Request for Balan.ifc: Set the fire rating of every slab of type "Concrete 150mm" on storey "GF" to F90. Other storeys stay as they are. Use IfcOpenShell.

First a look at what the model holds.

```python
import ifcopenshell
import ifcopenshell.util.element

model = ifcopenshell.open("Balan.ifc")
print(model.schema)
storey = next(s for s in model.by_type("IfcBuildingStorey") if s.Name == "GF")
slabs = [e for e in ifcopenshell.util.element.get_decomposition(storey) if e.is_a("IfcSlab")]
seen = {}
for e in slabs:
    element_type = ifcopenshell.util.element.get_type(e)
    key = (element_type.Name if element_type != e and element_type else None, ifcopenshell.util.element.get_pset(e, "Pset_SlabCommon", "FireRating"))
    seen[key] = seen.get(key, 0) + 1
for (name, value), count in sorted(seen.items(), key=str):
    print(count, "x", name, "|", value)
```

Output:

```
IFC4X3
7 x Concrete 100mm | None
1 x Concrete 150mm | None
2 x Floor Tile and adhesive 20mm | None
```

```python
import ifcopenshell
import ifcopenshell.api.pset
import ifcopenshell.util.element

model = ifcopenshell.open("Balan.ifc")

storey = next(s for s in model.by_type("IfcBuildingStorey") if s.Name == "GF")
slabs = [e for e in ifcopenshell.util.element.get_decomposition(storey) if e.is_a("IfcSlab")]

count = 0
for e in slabs:
    element_type = ifcopenshell.util.element.get_type(e)
    if element_type in (None, e) or element_type.Name != "Concrete 150mm":
        continue
    # add_pset returns the element's existing set when there is one.
    pset = ifcopenshell.api.pset.add_pset(model, product=e, name="Pset_SlabCommon")
    ifcopenshell.api.pset.edit_pset(model, pset=pset, properties={"FireRating": "F90"})
    count += 1

print(count, "slabs updated")

model.write("Balan_edited.ifc")
```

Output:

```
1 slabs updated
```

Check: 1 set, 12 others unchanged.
